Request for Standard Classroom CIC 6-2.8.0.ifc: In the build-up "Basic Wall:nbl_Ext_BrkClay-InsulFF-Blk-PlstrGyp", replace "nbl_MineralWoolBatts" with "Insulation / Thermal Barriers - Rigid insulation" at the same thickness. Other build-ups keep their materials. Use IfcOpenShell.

First a look at what the model holds.

```python
import ifcopenshell
import ifcopenshell.util.element

model = ifcopenshell.open("Standard Classroom CIC 6-2.8.0.ifc")
print(model.schema)
for layer_set in model.by_type("IfcMaterialLayerSet"):
    if layer_set.LayerSetName == "Basic Wall:nbl_Ext_BrkClay-InsulFF-Blk-PlstrGyp":
        for layer in layer_set.MaterialLayers:
            print(layer.id(), layer.Material and layer.Material.Name, layer.LayerThickness, sep=" | ")
        print(len(ifcopenshell.util.element.get_elements_by_material(model, layer_set)), "elements and types use it")
print(sorted(m.Name for m in model.by_type("IfcMaterial") if m.Name)[:60])
```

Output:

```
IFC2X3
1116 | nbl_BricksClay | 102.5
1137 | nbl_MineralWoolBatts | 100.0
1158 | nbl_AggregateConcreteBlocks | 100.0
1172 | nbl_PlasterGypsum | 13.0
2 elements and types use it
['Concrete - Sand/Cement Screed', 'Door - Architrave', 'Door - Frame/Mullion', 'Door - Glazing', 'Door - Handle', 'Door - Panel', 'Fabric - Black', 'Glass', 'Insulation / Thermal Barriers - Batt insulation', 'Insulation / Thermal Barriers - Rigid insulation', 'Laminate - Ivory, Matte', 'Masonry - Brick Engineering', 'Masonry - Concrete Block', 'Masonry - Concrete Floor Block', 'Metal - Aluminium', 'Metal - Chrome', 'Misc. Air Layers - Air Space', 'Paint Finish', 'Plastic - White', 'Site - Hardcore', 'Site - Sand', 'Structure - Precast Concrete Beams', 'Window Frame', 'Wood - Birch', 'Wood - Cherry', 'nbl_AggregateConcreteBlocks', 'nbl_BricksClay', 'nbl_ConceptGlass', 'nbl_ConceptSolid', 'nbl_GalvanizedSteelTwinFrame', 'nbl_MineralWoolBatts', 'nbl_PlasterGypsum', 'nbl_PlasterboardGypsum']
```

```python
import ifcopenshell
import ifcopenshell.api.material

model = ifcopenshell.open("Standard Classroom CIC 6-2.8.0.ifc")

layer_set = next(s for s in model.by_type("IfcMaterialLayerSet") if s.LayerSetName == "Basic Wall:nbl_Ext_BrkClay-InsulFF-Blk-PlstrGyp")
layer = next(l for l in layer_set.MaterialLayers if l.Material and l.Material.Name == "nbl_MineralWoolBatts")
material = next(m for m in model.by_type("IfcMaterial") if m.Name == "Insulation / Thermal Barriers - Rigid insulation")

# Point this one layer at the other material; renaming the old one would change it everywhere.
ifcopenshell.api.material.edit_layer(model, layer=layer, attributes={}, material=material)

print([l.Material.Name if l.Material else None for l in layer_set.MaterialLayers])

model.write("Standard Classroom CIC 6-2.8.0_edited.ifc")
```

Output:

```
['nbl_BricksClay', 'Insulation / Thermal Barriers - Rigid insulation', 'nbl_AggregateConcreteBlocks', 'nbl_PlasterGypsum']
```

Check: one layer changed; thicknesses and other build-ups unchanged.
